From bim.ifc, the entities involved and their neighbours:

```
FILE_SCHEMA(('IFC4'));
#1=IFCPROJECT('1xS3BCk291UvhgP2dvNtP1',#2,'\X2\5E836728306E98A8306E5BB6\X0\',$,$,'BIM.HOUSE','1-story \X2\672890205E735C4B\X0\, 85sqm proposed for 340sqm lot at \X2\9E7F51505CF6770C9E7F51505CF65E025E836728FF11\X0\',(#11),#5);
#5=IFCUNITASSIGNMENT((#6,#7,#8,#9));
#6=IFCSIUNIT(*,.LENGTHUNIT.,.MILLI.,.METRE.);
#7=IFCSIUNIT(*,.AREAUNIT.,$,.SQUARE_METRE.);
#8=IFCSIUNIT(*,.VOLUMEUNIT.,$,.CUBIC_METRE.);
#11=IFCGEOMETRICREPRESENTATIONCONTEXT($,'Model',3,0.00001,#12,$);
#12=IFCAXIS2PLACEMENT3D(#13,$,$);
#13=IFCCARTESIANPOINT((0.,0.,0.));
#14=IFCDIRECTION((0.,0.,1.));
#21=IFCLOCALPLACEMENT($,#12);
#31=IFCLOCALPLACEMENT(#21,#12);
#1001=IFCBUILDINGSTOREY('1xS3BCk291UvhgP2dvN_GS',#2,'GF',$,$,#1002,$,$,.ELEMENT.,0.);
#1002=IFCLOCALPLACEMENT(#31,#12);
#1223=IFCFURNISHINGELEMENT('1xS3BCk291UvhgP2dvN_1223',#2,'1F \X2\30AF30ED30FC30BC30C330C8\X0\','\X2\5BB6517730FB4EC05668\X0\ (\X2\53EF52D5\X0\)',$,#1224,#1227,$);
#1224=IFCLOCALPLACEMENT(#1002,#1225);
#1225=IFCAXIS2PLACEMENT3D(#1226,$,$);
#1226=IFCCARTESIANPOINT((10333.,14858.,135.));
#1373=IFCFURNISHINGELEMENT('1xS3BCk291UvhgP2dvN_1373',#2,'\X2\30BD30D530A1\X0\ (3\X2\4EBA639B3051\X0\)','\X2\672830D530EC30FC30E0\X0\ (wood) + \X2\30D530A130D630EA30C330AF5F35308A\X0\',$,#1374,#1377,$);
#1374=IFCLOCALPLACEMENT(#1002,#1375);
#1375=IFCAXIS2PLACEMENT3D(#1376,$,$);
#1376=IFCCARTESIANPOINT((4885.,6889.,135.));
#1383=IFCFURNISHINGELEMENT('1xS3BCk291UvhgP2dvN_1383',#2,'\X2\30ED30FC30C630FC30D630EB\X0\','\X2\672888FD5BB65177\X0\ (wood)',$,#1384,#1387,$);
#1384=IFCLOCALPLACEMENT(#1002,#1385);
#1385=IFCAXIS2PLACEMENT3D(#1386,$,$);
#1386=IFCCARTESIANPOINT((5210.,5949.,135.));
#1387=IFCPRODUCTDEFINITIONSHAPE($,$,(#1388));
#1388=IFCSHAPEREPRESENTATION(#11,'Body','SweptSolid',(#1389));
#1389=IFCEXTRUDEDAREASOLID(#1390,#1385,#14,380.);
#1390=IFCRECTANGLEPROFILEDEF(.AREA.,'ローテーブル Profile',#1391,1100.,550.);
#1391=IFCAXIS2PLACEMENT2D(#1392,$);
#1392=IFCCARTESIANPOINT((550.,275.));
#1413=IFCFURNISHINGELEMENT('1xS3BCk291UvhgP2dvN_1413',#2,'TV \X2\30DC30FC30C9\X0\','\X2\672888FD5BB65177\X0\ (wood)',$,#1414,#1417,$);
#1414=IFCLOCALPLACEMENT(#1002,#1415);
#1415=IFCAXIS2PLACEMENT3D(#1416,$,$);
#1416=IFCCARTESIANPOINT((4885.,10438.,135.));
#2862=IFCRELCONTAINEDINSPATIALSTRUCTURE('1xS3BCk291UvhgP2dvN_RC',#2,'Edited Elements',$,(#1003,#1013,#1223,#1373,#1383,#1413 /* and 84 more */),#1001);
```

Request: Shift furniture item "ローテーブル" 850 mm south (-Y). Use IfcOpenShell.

```python
import ifcopenshell
import ifcopenshell.api.geometry
import ifcopenshell.util.placement
import ifcopenshell.util.unit

model = ifcopenshell.open("bim.ifc")
unit_scale = ifcopenshell.util.unit.calculate_unit_scale(model)

item = model.by_id(1383)
matrix = ifcopenshell.util.placement.get_local_placement(item.ObjectPlacement)
matrix[1, 3] -= 0.85 / unit_scale
ifcopenshell.api.geometry.edit_object_placement(model, product=item, matrix=matrix, is_si=False)

print(ifcopenshell.util.placement.get_local_placement(item.ObjectPlacement).round(3) + 0.0)

model.write("bim_v2.ifc")
```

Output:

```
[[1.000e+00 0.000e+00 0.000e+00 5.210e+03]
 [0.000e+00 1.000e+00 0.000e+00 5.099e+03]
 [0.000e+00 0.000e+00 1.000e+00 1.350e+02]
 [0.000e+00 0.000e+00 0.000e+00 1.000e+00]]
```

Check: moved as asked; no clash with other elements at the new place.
